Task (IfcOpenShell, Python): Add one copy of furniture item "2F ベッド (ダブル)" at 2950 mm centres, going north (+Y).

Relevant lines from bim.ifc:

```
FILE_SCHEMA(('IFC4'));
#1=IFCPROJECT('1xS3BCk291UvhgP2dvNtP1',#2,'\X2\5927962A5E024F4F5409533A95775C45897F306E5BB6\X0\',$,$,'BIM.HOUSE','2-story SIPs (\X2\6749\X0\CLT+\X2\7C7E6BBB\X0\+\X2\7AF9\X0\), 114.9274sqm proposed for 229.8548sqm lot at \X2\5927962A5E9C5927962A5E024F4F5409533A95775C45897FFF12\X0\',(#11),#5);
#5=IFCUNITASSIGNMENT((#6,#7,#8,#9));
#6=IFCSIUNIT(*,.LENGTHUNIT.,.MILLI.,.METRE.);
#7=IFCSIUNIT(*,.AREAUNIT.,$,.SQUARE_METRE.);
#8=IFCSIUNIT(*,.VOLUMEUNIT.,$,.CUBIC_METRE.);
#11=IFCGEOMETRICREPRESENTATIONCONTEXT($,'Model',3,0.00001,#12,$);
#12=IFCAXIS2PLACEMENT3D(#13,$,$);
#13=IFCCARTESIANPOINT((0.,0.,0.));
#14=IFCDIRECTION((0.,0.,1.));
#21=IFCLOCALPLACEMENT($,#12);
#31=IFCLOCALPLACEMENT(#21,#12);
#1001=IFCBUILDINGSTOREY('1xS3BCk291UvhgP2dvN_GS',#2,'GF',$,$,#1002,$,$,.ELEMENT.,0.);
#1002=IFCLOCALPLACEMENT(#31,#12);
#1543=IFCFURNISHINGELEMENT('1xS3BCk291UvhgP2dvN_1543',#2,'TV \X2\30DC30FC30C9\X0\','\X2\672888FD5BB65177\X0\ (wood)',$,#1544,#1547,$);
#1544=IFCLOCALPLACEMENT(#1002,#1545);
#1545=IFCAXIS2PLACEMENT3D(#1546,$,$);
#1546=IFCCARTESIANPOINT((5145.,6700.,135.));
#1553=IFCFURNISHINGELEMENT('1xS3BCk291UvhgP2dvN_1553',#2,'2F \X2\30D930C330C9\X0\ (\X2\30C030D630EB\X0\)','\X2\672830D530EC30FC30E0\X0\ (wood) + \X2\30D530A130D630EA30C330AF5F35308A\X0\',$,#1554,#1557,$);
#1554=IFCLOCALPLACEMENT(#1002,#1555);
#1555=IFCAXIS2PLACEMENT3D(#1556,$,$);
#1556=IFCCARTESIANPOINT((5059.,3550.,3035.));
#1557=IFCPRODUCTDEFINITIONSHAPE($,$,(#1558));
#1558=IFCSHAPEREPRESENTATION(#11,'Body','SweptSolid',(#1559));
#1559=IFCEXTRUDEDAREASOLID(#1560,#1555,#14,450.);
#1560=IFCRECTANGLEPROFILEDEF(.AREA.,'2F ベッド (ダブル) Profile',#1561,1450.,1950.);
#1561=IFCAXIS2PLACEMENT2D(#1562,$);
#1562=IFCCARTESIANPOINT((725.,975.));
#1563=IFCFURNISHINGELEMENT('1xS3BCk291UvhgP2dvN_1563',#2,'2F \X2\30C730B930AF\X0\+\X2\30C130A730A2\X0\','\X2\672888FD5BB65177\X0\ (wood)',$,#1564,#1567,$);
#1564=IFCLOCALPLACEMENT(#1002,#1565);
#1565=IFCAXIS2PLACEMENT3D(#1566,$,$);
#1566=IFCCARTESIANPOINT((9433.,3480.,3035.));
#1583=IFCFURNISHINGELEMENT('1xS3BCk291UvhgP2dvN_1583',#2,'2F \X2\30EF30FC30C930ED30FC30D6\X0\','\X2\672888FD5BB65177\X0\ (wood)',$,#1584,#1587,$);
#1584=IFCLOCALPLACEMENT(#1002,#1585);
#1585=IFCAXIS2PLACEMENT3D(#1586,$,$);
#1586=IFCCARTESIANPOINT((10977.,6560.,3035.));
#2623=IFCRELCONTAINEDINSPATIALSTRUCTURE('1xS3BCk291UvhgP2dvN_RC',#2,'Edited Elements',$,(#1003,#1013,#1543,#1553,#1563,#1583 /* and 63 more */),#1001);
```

```python
import numpy as np
import ifcopenshell
import ifcopenshell.api.geometry
import ifcopenshell.api.root
import ifcopenshell.util.element
import ifcopenshell.util.placement
import ifcopenshell.util.unit

model = ifcopenshell.open("bim.ifc")
unit_scale = ifcopenshell.util.unit.calculate_unit_scale(model)


def reuse_history(source, copy):
    """copy_class also copies each property set's owner history, people and application; keep the originals."""
    for rel in copy.IsDefinedBy:
        if rel.is_a("IfcRelDefinesByProperties") and (history := rel.RelatingPropertyDefinition.OwnerHistory):
            rel.RelatingPropertyDefinition.OwnerHistory = source.OwnerHistory
            ifcopenshell.util.element.remove_deep2(model, history)


source = model.by_guid("1xS3BCk291UvhgP2dvN_1553")
base = ifcopenshell.util.placement.get_local_placement(source.ObjectPlacement)
step = np.array([0.0, 1.0, 0.0]) * 2.95 / unit_scale

for i in range(1, 2):
    copy = ifcopenshell.api.root.copy_class(model, product=source)
    copy.Representation = ifcopenshell.util.element.copy_deep(
        model, source.Representation, exclude=["IfcGeometricRepresentationContext", "IfcRepresentationMap"]
    )
    reuse_history(source, copy)
    matrix = base.copy()
    matrix[:3, 3] += i * step
    print("added at", matrix[:3, 3].round(3) + 0.0)
    ifcopenshell.api.geometry.edit_object_placement(model, product=copy, matrix=matrix, is_si=False)

model.write("bim_updated.ifc")
```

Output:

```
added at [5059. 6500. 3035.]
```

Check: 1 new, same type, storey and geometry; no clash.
